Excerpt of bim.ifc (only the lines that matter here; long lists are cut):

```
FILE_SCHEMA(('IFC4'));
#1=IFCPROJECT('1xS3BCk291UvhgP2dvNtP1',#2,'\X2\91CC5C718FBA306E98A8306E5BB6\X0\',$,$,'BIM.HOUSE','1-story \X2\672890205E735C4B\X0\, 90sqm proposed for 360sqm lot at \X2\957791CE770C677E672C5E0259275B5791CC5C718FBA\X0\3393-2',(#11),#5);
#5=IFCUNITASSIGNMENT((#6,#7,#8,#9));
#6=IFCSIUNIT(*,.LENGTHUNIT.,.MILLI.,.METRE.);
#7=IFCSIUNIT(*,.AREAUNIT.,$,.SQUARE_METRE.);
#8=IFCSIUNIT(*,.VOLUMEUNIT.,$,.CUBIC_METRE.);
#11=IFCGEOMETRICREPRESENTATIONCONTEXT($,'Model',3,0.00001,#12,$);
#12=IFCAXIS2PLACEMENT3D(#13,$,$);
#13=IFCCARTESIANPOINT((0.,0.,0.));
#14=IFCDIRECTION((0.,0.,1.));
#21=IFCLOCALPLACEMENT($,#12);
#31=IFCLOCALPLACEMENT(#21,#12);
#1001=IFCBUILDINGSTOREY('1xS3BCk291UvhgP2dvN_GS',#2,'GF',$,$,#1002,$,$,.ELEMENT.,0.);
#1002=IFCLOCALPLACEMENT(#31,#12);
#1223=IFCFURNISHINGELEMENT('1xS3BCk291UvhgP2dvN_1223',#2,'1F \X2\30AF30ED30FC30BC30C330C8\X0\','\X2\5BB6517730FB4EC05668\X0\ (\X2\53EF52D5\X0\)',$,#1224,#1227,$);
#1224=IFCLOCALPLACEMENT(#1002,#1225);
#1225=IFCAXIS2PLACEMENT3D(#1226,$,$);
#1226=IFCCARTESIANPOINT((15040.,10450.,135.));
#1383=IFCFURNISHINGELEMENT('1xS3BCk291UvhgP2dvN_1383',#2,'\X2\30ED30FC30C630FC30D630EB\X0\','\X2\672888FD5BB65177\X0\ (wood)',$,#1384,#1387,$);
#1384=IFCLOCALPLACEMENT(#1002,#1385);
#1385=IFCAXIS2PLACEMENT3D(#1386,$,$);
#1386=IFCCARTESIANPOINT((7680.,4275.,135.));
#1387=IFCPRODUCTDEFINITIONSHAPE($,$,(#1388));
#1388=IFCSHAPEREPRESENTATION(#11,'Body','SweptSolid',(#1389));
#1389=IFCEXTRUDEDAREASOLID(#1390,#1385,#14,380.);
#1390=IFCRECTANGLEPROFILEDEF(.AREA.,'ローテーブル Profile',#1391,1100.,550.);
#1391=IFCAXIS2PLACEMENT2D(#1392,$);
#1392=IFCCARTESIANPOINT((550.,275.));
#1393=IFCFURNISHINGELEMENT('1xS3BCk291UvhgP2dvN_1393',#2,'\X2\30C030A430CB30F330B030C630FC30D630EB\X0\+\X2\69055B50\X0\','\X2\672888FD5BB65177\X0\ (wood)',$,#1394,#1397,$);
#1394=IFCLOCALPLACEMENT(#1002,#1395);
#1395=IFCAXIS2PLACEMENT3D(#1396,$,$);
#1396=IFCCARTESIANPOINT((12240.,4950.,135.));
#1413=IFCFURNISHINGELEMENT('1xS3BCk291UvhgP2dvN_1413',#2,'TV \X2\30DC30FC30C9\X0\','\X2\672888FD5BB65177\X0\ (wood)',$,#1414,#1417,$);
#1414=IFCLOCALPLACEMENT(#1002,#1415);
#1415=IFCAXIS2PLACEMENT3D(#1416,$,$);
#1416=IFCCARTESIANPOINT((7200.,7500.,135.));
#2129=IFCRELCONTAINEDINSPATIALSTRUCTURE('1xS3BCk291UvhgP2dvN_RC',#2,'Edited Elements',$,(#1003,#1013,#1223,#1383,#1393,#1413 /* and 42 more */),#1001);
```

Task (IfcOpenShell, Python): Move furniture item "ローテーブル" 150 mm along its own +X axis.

```python
import ifcopenshell
import ifcopenshell.api.geometry
import ifcopenshell.util.placement

model = ifcopenshell.open("bim.ifc")

item = model.by_id(1383)
matrix = ifcopenshell.util.placement.get_local_placement(item.ObjectPlacement)
matrix[:3, 3] += matrix[:3, 0] * 150.0
ifcopenshell.api.geometry.edit_object_placement(model, product=item, matrix=matrix, is_si=False)

print(ifcopenshell.util.placement.get_local_placement(item.ObjectPlacement).round(3) + 0.0)

model.write("bim_v2.ifc")
```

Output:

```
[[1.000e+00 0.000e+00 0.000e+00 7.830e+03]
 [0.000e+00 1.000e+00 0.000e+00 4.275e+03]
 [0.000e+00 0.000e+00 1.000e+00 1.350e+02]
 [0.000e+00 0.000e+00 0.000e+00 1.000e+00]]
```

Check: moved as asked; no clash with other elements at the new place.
